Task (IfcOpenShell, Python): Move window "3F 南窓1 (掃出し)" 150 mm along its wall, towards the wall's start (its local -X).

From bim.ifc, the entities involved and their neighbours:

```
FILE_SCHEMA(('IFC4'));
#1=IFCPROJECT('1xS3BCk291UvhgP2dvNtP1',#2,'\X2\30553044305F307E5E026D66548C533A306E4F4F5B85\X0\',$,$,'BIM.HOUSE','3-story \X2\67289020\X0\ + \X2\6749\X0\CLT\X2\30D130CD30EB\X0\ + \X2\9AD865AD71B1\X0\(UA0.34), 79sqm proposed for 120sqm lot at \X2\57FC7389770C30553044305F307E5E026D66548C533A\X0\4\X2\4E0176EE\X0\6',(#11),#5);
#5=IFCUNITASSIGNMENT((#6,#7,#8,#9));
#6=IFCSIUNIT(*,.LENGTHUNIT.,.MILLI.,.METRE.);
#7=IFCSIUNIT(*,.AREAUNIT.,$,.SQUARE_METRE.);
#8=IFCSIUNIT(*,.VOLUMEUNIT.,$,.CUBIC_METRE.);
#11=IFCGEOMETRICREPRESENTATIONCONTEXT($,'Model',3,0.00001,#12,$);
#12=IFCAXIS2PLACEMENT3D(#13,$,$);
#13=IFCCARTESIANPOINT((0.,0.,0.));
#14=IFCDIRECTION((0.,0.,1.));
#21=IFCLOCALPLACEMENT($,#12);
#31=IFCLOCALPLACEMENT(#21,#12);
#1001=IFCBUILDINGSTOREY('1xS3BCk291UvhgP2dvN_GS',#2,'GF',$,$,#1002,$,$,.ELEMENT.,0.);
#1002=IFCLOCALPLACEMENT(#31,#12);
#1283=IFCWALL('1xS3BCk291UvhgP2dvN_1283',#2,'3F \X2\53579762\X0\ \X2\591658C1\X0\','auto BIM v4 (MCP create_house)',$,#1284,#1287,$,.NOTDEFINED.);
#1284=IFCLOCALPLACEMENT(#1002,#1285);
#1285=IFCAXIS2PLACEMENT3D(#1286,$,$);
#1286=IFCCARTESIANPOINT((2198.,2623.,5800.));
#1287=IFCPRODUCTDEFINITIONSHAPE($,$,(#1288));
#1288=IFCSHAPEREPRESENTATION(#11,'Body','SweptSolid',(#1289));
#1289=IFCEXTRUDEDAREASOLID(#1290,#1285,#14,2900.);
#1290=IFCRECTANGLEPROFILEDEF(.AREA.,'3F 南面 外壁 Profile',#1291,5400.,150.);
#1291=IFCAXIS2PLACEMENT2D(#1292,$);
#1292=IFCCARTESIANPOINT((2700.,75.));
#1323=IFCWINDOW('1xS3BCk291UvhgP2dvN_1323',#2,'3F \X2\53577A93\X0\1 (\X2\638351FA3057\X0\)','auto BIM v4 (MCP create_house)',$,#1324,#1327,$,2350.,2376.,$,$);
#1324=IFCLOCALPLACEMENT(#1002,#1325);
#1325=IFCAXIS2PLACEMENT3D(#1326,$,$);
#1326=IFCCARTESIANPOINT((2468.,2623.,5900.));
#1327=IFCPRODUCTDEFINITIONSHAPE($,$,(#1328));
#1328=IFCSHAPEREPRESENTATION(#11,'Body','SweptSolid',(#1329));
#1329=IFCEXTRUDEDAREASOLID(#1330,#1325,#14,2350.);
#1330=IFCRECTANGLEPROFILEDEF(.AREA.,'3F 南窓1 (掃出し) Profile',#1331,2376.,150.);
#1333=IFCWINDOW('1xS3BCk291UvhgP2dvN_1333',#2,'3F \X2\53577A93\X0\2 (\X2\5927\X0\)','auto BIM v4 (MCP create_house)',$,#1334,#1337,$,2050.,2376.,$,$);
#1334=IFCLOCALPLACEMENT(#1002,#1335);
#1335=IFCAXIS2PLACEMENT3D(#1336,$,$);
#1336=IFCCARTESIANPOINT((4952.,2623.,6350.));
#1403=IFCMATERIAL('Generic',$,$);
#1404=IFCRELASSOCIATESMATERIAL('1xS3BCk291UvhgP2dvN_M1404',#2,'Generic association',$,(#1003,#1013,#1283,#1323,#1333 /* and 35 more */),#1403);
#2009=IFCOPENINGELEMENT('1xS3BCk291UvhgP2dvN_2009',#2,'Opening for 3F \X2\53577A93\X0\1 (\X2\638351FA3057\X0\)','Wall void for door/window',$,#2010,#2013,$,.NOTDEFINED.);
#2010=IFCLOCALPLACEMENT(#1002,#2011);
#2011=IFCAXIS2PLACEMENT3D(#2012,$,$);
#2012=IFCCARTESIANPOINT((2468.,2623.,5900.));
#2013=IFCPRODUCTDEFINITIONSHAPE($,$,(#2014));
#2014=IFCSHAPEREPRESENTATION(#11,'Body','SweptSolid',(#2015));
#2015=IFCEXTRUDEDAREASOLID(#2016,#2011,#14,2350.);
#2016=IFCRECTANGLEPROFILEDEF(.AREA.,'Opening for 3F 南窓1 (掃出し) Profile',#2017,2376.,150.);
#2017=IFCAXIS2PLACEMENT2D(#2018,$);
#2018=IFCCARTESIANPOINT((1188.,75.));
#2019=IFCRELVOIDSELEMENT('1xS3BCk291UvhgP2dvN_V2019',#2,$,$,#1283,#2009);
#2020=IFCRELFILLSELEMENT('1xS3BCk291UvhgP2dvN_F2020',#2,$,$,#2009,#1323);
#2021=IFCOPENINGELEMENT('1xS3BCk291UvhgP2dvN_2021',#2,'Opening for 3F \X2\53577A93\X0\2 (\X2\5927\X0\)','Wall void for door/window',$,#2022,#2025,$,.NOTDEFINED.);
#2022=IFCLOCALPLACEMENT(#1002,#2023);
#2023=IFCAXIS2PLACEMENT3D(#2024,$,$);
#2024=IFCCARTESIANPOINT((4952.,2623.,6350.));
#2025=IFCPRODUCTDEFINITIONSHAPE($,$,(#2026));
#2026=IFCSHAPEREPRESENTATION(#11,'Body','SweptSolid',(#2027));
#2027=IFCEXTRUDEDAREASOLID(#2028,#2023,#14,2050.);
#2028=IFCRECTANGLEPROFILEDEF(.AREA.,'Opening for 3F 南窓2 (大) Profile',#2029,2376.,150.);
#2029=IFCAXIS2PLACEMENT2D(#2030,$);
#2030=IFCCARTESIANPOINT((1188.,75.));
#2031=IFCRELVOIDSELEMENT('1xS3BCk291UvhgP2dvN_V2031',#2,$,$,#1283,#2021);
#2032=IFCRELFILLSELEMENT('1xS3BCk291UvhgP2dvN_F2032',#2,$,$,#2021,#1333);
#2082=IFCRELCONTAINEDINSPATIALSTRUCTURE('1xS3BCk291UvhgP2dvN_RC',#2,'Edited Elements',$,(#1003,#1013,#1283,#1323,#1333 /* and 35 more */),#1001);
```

```python
import ifcopenshell
import ifcopenshell.api.geometry
import ifcopenshell.util.placement
import ifcopenshell.util.unit

model = ifcopenshell.open("bim.ifc")
unit_scale = ifcopenshell.util.unit.calculate_unit_scale(model)

window = model.by_guid("1xS3BCk291UvhgP2dvN_1323")
opening = window.FillsVoids[0].RelatingOpeningElement
wall = opening.VoidsElements[0].RelatingBuildingElement

wall_matrix = ifcopenshell.util.placement.get_local_placement(wall.ObjectPlacement)
shift = wall_matrix[:3, 0] * -0.15 / unit_scale
before = ifcopenshell.util.placement.get_local_placement(window.ObjectPlacement)[:3, 3].copy()

# The window is not placed relative to its opening, so move both.
for product in (opening, window):
    matrix = ifcopenshell.util.placement.get_local_placement(product.ObjectPlacement)
    matrix[:3, 3] += shift
    ifcopenshell.api.geometry.edit_object_placement(model, product=product, matrix=matrix, is_si=False)

after = ifcopenshell.util.placement.get_local_placement(window.ObjectPlacement)[:3, 3]
print("window moved by", (after - before).round(3) + 0.0)

model.write("bim_edited.ifc")
```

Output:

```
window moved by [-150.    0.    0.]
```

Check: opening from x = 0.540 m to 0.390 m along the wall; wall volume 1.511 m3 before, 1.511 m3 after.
